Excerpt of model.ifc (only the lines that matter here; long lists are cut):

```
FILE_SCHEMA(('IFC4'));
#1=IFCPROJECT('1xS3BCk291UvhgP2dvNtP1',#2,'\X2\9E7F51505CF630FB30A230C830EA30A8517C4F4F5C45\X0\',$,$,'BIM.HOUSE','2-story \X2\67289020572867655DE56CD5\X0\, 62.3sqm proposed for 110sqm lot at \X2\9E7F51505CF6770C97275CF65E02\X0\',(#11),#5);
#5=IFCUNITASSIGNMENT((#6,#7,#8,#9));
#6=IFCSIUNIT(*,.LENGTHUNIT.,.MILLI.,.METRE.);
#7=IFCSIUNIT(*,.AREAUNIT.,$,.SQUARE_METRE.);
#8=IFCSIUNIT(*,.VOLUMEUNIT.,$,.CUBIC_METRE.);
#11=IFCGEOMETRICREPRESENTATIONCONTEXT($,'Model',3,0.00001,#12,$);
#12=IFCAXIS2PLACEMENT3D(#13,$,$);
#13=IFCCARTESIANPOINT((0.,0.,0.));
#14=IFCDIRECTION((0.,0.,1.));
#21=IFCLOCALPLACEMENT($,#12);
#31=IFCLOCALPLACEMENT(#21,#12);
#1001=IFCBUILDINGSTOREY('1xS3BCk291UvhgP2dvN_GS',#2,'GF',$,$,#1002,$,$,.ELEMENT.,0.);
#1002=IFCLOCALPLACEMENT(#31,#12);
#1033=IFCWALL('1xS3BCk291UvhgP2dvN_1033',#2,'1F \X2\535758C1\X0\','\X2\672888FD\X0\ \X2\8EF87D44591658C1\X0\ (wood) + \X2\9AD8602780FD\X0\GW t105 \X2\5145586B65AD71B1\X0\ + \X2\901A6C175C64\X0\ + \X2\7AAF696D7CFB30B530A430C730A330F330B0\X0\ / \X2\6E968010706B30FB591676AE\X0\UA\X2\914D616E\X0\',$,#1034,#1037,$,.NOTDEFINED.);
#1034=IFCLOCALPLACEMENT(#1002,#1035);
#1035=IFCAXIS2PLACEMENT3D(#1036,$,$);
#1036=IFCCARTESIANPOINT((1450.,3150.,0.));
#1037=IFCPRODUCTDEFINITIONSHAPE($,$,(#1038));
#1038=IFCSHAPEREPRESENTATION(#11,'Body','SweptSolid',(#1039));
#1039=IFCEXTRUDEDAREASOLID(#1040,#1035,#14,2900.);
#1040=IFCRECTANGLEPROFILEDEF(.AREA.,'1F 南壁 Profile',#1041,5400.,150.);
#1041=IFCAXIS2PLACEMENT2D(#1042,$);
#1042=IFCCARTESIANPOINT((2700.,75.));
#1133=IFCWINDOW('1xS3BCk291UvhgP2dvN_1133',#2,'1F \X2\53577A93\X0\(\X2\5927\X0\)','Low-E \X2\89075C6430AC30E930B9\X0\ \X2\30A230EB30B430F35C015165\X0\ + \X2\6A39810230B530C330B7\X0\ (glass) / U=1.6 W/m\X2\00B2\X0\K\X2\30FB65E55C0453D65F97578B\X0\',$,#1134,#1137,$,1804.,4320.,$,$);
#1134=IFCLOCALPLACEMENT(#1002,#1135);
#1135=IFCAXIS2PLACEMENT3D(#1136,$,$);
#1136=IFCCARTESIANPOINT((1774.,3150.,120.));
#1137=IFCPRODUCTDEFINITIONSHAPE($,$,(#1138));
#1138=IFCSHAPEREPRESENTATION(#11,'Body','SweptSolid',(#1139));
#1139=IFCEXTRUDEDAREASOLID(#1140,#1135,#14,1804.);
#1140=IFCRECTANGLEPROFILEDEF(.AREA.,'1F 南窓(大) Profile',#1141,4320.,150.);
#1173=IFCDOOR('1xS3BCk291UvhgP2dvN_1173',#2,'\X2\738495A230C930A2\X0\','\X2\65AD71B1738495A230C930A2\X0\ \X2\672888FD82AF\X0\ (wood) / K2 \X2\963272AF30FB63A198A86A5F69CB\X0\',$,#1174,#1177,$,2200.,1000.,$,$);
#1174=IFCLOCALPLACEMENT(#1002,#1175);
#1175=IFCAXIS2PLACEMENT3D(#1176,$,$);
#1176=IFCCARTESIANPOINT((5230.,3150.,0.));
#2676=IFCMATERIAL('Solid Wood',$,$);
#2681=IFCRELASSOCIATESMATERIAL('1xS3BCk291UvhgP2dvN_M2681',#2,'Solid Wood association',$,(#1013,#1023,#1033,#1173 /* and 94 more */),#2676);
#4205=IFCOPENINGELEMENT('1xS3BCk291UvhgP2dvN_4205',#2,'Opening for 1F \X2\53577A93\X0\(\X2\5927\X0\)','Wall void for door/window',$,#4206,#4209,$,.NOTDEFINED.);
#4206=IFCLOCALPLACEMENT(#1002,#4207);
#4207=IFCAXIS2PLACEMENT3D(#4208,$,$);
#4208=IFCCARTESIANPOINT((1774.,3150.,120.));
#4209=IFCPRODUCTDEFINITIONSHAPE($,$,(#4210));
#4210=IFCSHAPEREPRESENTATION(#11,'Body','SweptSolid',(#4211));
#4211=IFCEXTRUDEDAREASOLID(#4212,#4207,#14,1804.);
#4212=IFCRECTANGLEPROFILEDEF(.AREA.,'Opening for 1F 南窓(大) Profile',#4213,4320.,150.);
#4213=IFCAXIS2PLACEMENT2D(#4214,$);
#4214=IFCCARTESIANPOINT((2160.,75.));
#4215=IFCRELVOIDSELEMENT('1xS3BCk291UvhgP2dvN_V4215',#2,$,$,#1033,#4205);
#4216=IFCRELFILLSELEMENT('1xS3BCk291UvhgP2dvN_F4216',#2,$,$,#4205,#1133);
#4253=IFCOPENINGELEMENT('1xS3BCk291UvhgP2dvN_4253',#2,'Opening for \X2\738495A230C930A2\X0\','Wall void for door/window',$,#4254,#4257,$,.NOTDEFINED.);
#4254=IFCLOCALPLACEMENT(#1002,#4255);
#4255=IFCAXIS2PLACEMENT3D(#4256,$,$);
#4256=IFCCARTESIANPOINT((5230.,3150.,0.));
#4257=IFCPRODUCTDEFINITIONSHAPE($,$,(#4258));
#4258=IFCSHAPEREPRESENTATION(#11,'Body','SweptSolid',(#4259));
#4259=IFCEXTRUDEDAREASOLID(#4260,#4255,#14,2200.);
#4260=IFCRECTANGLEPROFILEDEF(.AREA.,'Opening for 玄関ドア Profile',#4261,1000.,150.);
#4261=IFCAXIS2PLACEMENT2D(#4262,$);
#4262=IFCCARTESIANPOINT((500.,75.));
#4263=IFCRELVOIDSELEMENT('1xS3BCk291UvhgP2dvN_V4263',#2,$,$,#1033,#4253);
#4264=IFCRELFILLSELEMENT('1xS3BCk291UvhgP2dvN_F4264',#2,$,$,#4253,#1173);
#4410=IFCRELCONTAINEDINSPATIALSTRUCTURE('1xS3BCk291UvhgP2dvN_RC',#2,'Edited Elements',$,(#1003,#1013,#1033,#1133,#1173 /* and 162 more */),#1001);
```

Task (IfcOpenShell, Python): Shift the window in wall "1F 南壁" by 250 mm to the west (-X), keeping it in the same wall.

```python
import ifcopenshell
import ifcopenshell.api.geometry
import ifcopenshell.util.placement
import ifcopenshell.util.unit

model = ifcopenshell.open("model.ifc")
unit_scale = ifcopenshell.util.unit.calculate_unit_scale(model)

window = model.by_guid("1xS3BCk291UvhgP2dvN_1133")
opening = window.FillsVoids[0].RelatingOpeningElement
wall = opening.VoidsElements[0].RelatingBuildingElement

wall_matrix = ifcopenshell.util.placement.get_local_placement(wall.ObjectPlacement)
shift = wall_matrix[:3, 0] * -0.25 / unit_scale
before = ifcopenshell.util.placement.get_local_placement(window.ObjectPlacement)[:3, 3].copy()

# The window is not placed relative to its opening, so move both.
for product in (opening, window):
    matrix = ifcopenshell.util.placement.get_local_placement(product.ObjectPlacement)
    matrix[:3, 3] += shift
    ifcopenshell.api.geometry.edit_object_placement(model, product=product, matrix=matrix, is_si=False)

after = ifcopenshell.util.placement.get_local_placement(window.ObjectPlacement)[:3, 3]
print("window moved by", (after - before).round(3) + 0.0)

model.write("model_rev.ifc")
```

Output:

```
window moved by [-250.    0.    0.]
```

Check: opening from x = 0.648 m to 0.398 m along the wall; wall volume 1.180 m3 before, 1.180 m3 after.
